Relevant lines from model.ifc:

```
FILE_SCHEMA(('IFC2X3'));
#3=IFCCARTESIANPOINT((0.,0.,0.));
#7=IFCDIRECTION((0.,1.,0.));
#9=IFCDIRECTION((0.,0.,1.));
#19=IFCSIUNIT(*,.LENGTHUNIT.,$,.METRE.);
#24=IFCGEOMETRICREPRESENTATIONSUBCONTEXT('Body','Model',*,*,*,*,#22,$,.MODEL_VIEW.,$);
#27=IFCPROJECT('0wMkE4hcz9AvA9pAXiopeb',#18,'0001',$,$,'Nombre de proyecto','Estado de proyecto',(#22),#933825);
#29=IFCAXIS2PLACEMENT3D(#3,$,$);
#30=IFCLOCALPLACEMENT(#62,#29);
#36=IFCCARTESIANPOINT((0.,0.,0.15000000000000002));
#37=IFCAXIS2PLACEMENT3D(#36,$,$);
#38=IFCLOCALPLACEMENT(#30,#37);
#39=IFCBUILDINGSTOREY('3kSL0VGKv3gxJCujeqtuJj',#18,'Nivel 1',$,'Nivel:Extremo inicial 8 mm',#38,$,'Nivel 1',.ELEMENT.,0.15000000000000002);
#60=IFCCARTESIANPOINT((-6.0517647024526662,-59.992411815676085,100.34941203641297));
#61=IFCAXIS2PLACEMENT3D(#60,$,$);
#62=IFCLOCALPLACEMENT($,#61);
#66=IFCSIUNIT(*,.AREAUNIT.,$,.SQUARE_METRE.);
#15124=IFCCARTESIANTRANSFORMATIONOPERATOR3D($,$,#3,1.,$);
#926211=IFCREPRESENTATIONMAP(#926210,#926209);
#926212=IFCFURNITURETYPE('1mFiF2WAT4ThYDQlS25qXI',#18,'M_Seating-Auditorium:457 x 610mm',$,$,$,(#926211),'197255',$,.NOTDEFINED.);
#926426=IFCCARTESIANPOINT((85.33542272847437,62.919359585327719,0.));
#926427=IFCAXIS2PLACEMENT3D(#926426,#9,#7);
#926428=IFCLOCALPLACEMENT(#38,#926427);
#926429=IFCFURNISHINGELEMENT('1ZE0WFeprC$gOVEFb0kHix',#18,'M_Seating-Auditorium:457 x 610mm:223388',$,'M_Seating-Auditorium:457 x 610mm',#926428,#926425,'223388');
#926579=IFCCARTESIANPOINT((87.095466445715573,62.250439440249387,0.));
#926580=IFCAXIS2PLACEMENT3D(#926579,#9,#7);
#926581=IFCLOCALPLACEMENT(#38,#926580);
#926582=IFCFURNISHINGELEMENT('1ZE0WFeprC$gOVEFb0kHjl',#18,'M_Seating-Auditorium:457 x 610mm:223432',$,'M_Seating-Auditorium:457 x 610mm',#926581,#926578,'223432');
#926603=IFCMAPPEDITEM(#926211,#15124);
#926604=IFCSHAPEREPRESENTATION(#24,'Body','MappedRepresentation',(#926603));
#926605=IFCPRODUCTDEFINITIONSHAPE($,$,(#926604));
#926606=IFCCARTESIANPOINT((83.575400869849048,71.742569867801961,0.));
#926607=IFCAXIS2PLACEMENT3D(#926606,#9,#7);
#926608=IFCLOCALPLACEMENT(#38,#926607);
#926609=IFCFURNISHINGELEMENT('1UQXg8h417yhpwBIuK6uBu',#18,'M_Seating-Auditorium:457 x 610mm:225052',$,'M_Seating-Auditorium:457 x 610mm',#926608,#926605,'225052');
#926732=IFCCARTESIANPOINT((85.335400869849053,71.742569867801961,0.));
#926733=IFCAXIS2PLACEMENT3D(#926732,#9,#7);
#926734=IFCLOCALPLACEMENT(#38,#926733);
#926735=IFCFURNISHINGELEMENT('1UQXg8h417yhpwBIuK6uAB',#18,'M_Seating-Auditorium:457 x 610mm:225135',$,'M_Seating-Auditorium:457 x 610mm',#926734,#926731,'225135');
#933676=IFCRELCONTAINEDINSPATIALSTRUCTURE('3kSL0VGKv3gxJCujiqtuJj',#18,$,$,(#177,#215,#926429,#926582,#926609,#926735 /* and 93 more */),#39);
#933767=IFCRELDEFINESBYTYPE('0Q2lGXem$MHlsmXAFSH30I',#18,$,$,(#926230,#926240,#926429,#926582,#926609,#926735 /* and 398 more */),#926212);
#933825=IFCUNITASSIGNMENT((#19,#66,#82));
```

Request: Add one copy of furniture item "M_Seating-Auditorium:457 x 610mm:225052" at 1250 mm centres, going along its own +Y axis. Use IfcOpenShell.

```python
import ifcopenshell
import ifcopenshell.api.geometry
import ifcopenshell.api.root
import ifcopenshell.util.element
import ifcopenshell.util.placement

model = ifcopenshell.open("model.ifc")


def reuse_history(source, copy):
    """copy_class also copies each property set's owner history, people and application; keep the originals."""
    for rel in copy.IsDefinedBy:
        if rel.is_a("IfcRelDefinesByProperties") and (history := rel.RelatingPropertyDefinition.OwnerHistory):
            rel.RelatingPropertyDefinition.OwnerHistory = source.OwnerHistory
            ifcopenshell.util.element.remove_deep2(model, history)


source = model.by_guid("1UQXg8h417yhpwBIuK6uBu")
base = ifcopenshell.util.placement.get_local_placement(source.ObjectPlacement)
step = base[:3, 1] * 1.25

for i in range(1, 2):
    copy = ifcopenshell.api.root.copy_class(model, product=source)
    copy.Representation = ifcopenshell.util.element.copy_deep(
        model, source.Representation, exclude=["IfcGeometricRepresentationContext", "IfcRepresentationMap"]
    )
    copy.Name = "M_Seating-Auditorium:457 x 610mm"
    copy.Tag = None
    reuse_history(source, copy)
    matrix = base.copy()
    matrix[:3, 3] += i * step
    print("added at", matrix[:3, 3].round(3) + 0.0)
    ifcopenshell.api.geometry.edit_object_placement(model, product=copy, matrix=matrix, is_si=False)

model.write("model-out.ifc")
```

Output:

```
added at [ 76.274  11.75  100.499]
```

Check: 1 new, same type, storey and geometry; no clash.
